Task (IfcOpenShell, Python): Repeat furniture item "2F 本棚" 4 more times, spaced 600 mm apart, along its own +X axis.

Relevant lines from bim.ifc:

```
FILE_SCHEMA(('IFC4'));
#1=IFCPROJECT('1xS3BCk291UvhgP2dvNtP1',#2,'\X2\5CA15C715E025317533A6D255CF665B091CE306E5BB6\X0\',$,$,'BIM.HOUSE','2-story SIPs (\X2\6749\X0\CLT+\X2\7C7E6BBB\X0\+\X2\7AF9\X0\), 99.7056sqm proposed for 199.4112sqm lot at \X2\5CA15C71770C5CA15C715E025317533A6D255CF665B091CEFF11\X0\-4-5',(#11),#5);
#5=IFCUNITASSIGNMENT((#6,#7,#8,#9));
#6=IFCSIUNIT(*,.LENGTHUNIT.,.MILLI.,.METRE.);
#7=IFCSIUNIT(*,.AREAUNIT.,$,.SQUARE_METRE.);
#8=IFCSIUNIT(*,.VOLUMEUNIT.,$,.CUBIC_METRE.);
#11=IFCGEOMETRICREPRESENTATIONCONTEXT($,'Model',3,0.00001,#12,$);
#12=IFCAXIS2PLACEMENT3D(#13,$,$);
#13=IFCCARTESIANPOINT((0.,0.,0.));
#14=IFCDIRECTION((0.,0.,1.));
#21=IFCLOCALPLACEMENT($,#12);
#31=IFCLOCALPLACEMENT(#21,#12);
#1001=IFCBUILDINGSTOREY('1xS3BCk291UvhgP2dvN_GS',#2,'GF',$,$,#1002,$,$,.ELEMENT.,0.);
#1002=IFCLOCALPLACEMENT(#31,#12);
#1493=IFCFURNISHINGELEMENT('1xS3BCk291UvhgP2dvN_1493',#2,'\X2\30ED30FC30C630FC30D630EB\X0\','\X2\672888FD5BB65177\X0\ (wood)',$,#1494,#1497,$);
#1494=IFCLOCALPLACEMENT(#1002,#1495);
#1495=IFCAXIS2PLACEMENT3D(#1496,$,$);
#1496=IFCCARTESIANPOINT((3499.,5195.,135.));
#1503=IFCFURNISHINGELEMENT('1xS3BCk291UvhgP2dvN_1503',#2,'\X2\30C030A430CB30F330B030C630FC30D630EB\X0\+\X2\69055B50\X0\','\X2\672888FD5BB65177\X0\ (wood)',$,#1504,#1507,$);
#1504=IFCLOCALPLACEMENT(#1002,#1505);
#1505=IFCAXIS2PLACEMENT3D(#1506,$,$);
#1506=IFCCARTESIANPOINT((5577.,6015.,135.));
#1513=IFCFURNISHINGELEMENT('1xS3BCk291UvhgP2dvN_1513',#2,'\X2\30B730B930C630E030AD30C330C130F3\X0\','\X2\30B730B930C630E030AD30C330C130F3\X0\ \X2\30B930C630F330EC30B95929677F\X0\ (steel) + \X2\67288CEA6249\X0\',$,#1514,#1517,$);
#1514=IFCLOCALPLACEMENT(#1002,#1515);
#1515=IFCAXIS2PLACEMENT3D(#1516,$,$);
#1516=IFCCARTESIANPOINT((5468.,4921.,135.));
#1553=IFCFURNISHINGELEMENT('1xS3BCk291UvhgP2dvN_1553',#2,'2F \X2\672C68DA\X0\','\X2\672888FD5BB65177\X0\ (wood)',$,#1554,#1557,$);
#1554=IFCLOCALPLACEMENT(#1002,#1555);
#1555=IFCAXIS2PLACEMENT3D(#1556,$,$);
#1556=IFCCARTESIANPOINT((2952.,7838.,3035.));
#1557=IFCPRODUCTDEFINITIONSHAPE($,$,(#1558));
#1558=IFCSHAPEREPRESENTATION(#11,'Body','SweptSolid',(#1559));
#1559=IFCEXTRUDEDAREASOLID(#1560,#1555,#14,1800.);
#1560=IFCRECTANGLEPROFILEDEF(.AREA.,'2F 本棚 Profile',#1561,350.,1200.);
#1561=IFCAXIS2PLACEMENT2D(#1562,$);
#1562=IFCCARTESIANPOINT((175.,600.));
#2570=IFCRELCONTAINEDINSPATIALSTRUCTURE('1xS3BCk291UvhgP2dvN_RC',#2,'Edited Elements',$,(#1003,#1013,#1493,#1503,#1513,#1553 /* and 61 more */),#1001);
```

```python
import ifcopenshell
import ifcopenshell.api.geometry
import ifcopenshell.api.root
import ifcopenshell.util.element
import ifcopenshell.util.placement

model = ifcopenshell.open("bim.ifc")


def reuse_history(source, copy):
    """copy_class also copies each property set's owner history, people and application; keep the originals."""
    for rel in copy.IsDefinedBy:
        if rel.is_a("IfcRelDefinesByProperties") and (history := rel.RelatingPropertyDefinition.OwnerHistory):
            rel.RelatingPropertyDefinition.OwnerHistory = source.OwnerHistory
            ifcopenshell.util.element.remove_deep2(model, history)


source = model.by_guid("1xS3BCk291UvhgP2dvN_1553")
base = ifcopenshell.util.placement.get_local_placement(source.ObjectPlacement)
step = base[:3, 0] * 600.0

for i in range(1, 5):
    copy = ifcopenshell.api.root.copy_class(model, product=source)
    copy.Representation = ifcopenshell.util.element.copy_deep(
        model, source.Representation, exclude=["IfcGeometricRepresentationContext", "IfcRepresentationMap"]
    )
    reuse_history(source, copy)
    matrix = base.copy()
    matrix[:3, 3] += i * step
    print("added at", matrix[:3, 3].round(3) + 0.0)
    ifcopenshell.api.geometry.edit_object_placement(model, product=copy, matrix=matrix, is_si=False)

model.write("bim_v2.ifc")
```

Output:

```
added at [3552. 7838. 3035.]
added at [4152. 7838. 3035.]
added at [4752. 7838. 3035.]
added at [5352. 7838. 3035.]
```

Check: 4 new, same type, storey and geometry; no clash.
